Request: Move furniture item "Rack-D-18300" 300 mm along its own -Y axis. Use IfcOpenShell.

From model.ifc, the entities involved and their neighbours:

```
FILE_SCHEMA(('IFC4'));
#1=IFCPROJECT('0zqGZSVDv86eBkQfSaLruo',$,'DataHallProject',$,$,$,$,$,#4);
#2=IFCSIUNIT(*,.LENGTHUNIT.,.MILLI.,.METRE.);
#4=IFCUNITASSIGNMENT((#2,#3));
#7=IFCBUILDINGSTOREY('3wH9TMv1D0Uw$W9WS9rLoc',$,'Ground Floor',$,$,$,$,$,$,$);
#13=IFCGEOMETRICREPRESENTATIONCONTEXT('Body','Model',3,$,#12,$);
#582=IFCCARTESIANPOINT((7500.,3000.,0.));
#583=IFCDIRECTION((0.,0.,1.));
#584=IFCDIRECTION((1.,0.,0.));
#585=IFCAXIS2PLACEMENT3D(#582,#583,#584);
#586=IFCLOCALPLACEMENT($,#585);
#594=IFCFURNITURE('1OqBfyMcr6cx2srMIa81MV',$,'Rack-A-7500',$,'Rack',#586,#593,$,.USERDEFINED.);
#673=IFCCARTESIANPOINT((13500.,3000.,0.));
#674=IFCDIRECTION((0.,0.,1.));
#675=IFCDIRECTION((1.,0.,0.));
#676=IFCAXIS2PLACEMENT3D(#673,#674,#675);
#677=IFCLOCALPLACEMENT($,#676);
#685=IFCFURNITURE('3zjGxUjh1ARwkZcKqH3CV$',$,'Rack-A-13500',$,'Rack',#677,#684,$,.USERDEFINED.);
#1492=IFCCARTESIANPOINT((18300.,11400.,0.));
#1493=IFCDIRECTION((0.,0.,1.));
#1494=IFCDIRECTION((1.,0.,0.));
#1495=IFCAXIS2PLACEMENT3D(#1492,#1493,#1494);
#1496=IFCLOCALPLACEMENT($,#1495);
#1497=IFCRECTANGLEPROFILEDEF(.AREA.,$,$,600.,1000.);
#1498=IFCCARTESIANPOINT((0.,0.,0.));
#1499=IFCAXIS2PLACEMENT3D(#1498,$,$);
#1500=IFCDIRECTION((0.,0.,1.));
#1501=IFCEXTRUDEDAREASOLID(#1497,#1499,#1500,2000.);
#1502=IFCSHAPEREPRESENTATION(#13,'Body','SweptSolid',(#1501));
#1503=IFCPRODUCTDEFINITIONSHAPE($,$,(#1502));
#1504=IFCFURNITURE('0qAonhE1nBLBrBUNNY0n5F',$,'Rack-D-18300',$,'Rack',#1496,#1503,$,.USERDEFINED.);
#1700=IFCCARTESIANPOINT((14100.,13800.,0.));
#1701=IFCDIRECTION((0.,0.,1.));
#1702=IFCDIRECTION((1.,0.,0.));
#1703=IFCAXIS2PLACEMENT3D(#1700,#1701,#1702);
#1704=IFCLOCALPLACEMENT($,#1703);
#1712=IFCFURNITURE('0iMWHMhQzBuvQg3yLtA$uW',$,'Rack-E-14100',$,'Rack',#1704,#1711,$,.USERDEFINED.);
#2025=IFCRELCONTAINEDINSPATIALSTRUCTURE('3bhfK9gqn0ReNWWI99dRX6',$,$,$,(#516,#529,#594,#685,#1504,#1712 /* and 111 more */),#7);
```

```python
import ifcopenshell
import ifcopenshell.api.geometry
import ifcopenshell.util.placement

model = ifcopenshell.open("model.ifc")

item = model.by_guid("0qAonhE1nBLBrBUNNY0n5F")
matrix = ifcopenshell.util.placement.get_local_placement(item.ObjectPlacement)
matrix[:3, 3] -= matrix[:3, 1] * 300.0
ifcopenshell.api.geometry.edit_object_placement(model, product=item, matrix=matrix, is_si=False)

print(ifcopenshell.util.placement.get_local_placement(item.ObjectPlacement).round(3) + 0.0)

model.write("model_rev.ifc")
```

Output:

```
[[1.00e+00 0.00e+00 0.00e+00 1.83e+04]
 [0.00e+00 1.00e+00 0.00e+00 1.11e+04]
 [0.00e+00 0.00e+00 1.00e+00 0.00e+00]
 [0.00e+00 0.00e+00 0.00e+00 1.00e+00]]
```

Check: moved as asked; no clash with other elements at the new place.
